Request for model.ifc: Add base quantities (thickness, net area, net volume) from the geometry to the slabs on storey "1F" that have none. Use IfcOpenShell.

First a look at what the model holds.

```python
import ifcopenshell
import ifcopenshell.util.element
import ifcopenshell.util.unit

model = ifcopenshell.open("model.ifc")
print(model.schema)
for unit_type in ("LENGTHUNIT", "AREAUNIT", "VOLUMEUNIT"):
    print(unit_type, ifcopenshell.util.unit.calculate_unit_scale(model, unit_type))
storey = next(s for s in model.by_type("IfcBuildingStorey") if s.Name == "1F")
slabs = [e for e in ifcopenshell.util.element.get_decomposition(storey) if e.is_a("IfcSlab")]
for e in sorted(slabs, key=lambda e: e.id()):
    print(e.id(), e.is_a(), e.Name, list(ifcopenshell.util.element.get_psets(e, qtos_only=True)), sep=" | ")
```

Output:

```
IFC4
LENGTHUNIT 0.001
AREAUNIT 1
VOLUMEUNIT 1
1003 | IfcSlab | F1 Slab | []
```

```python
import ifcopenshell
import ifcopenshell.api.pset
import ifcopenshell.geom
import ifcopenshell.util.element
import ifcopenshell.util.shape
import ifcopenshell.util.unit

model = ifcopenshell.open("model.ifc")
unit_scale = ifcopenshell.util.unit.calculate_unit_scale(model)
area_scale = ifcopenshell.util.unit.calculate_unit_scale(model, "AREAUNIT")
volume_scale = ifcopenshell.util.unit.calculate_unit_scale(model, "VOLUMEUNIT")
settings = ifcopenshell.geom.settings()

storey = next(s for s in model.by_type("IfcBuildingStorey") if s.Name == "1F")
slabs = [e for e in ifcopenshell.util.element.get_decomposition(storey) if e.is_a("IfcSlab")]

for e in sorted(slabs, key=lambda e: e.id()):
    if ifcopenshell.util.element.get_psets(e, qtos_only=True, should_inherit=False):
        continue
    # Geometry comes back in metres, in the element's own axes.
    shape = ifcopenshell.geom.create_shape(settings, e)
    values = {
        "Width": ifcopenshell.util.shape.get_z(shape.geometry) / unit_scale,
        "NetArea": ifcopenshell.util.shape.get_footprint_area(shape.geometry) / area_scale,
        "NetVolume": ifcopenshell.util.shape.get_volume(shape.geometry) / volume_scale,
    }
    qto = ifcopenshell.api.pset.add_qto(model, product=e, name="Qto_SlabBaseQuantities")
    ifcopenshell.api.pset.edit_qto(model, qto=qto, properties=values)
    print(e.id(), {k: round(v, 3) for k, v in values.items()})

model.write("model_rev.ifc")
```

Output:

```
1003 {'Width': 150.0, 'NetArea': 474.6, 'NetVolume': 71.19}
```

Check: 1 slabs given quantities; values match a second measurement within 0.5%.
